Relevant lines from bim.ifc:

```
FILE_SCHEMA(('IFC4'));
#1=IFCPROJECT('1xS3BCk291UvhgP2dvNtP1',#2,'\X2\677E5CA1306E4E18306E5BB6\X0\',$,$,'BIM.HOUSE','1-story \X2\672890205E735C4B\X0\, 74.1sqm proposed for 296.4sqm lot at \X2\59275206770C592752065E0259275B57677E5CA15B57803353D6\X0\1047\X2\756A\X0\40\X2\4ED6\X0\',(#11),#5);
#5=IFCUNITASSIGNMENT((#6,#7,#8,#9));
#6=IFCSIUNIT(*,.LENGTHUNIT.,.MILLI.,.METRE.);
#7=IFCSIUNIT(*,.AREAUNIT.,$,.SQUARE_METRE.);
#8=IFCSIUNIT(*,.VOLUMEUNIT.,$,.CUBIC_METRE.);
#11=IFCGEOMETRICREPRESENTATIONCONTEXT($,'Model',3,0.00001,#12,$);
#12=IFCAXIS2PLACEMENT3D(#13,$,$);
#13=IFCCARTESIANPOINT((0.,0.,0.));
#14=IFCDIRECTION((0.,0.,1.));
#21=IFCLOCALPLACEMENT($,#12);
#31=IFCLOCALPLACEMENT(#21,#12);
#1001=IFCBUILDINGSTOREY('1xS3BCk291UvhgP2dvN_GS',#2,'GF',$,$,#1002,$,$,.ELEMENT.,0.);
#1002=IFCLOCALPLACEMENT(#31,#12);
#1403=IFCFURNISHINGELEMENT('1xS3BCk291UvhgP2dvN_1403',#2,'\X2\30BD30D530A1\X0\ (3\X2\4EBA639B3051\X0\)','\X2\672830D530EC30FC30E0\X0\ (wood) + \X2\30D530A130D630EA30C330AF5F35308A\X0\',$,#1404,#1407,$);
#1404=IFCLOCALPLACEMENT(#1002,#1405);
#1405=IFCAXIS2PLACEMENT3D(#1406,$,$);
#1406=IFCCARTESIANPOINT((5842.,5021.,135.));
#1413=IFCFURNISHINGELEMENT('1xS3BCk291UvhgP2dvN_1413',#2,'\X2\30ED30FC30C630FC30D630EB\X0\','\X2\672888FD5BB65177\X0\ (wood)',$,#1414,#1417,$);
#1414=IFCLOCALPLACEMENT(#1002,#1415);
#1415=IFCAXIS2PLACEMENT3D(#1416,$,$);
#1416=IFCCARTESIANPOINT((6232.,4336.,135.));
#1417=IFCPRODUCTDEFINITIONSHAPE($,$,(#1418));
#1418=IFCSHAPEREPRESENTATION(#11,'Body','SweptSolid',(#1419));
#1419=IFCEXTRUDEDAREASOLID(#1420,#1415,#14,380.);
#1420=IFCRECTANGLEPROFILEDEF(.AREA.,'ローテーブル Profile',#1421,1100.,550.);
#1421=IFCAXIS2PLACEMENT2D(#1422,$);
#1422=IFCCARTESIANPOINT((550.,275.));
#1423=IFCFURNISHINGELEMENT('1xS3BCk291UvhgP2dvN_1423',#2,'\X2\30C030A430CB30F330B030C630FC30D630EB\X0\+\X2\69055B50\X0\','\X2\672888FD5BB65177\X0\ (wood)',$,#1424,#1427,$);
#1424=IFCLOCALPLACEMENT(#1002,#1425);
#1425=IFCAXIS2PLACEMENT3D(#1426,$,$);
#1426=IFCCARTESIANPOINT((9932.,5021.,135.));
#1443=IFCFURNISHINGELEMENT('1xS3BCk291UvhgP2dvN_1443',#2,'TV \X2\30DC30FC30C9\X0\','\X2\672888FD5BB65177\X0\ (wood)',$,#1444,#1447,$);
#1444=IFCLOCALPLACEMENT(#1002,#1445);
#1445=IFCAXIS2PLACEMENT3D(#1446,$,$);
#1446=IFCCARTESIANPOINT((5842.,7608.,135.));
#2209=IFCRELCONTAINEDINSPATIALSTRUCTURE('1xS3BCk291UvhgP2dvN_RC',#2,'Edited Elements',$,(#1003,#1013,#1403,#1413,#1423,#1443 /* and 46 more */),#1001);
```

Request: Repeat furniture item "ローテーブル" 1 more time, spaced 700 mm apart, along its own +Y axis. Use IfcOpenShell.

```python
import ifcopenshell
import ifcopenshell.api.geometry
import ifcopenshell.api.root
import ifcopenshell.util.element
import ifcopenshell.util.placement

model = ifcopenshell.open("bim.ifc")


def reuse_history(source, copy):
    """copy_class also copies each property set's owner history, people and application; keep the originals."""
    for rel in copy.IsDefinedBy:
        if rel.is_a("IfcRelDefinesByProperties") and (history := rel.RelatingPropertyDefinition.OwnerHistory):
            rel.RelatingPropertyDefinition.OwnerHistory = source.OwnerHistory
            ifcopenshell.util.element.remove_deep2(model, history)


source = model.by_id(1413)
base = ifcopenshell.util.placement.get_local_placement(source.ObjectPlacement)
step = base[:3, 1] * 700.0

for i in range(1, 2):
    copy = ifcopenshell.api.root.copy_class(model, product=source)
    copy.Representation = ifcopenshell.util.element.copy_deep(
        model, source.Representation, exclude=["IfcGeometricRepresentationContext", "IfcRepresentationMap"]
    )
    reuse_history(source, copy)
    matrix = base.copy()
    matrix[:3, 3] += i * step
    print("added at", matrix[:3, 3].round(3) + 0.0)
    ifcopenshell.api.geometry.edit_object_placement(model, product=copy, matrix=matrix, is_si=False)

model.write("bim_v2.ifc")
```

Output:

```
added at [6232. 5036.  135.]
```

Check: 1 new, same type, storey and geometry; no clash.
